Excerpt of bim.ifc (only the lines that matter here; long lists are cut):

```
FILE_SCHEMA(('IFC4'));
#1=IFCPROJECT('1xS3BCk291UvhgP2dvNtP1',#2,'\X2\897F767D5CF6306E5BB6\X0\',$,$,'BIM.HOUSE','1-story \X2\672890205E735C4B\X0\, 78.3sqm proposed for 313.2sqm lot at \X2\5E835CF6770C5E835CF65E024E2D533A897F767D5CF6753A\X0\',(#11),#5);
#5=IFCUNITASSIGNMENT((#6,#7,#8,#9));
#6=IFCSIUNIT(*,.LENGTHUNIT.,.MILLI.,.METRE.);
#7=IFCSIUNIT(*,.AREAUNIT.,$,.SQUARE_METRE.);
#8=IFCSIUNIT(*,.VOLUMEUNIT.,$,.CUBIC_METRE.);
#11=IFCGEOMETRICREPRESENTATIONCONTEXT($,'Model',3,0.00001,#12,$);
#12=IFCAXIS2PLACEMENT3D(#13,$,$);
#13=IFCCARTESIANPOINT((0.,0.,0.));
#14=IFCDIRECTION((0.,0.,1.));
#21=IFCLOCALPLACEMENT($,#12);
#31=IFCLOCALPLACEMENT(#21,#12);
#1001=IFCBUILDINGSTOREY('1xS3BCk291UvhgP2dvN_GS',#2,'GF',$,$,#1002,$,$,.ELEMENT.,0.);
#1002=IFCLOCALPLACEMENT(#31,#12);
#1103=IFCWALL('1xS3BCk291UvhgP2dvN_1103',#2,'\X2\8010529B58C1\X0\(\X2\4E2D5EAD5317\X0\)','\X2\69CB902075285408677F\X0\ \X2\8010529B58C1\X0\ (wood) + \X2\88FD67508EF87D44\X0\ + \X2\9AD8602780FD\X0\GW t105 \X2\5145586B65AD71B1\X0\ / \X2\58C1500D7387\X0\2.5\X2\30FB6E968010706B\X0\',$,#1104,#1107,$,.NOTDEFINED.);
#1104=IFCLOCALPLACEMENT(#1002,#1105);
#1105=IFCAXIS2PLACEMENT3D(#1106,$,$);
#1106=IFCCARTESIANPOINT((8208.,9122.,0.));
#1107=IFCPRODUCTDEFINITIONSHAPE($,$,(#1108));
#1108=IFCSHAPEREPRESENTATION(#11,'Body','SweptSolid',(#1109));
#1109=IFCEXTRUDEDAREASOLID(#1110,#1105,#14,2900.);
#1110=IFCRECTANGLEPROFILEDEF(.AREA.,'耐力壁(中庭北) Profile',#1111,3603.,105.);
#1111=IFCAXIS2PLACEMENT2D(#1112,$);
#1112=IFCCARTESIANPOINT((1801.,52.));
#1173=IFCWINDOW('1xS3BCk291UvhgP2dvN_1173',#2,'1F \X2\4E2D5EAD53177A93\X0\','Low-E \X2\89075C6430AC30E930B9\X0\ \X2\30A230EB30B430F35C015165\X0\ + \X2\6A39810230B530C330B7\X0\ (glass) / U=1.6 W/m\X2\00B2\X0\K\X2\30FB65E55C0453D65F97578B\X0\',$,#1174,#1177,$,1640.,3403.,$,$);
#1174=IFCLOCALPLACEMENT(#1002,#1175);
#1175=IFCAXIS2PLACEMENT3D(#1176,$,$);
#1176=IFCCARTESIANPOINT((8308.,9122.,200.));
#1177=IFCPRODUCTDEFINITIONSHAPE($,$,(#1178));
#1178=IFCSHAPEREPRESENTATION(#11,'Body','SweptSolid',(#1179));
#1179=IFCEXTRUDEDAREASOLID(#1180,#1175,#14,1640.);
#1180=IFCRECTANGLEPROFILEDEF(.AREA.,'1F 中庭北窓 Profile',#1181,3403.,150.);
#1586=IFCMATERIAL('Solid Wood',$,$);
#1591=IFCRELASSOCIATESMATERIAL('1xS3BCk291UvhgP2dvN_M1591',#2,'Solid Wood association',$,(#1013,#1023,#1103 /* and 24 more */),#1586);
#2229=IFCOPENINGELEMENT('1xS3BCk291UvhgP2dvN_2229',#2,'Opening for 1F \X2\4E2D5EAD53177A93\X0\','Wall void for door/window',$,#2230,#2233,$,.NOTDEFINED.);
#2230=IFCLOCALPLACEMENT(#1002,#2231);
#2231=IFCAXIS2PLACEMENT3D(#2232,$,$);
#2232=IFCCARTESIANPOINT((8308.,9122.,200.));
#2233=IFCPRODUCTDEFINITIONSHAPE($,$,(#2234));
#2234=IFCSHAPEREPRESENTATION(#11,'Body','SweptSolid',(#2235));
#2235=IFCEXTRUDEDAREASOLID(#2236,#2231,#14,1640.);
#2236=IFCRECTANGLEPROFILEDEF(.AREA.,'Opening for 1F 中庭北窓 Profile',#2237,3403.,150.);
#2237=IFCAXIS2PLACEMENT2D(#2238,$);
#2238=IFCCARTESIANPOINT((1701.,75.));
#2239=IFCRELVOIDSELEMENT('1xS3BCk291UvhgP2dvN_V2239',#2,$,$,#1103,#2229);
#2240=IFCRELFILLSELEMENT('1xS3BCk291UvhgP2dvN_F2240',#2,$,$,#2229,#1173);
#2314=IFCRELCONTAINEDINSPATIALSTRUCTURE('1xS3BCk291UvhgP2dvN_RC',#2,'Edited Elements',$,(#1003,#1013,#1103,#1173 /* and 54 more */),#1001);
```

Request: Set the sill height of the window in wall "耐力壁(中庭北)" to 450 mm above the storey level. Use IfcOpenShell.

```python
import numpy as np
import ifcopenshell
import ifcopenshell.api.geometry
import ifcopenshell.geom
import ifcopenshell.util.element
import ifcopenshell.util.placement
import ifcopenshell.util.shape
import ifcopenshell.util.unit

model = ifcopenshell.open("bim.ifc")
unit_scale = ifcopenshell.util.unit.calculate_unit_scale(model)

window = model.by_id(1173)
opening = window.FillsVoids[0].RelatingOpeningElement
storey = ifcopenshell.util.element.get_container(window, ifc_class="IfcBuildingStorey")
level = ifcopenshell.util.placement.get_local_placement(storey.ObjectPlacement)[2, 3]

# The opening's origin need not be at the sill, so measure its lowest point.
shape = ifcopenshell.geom.create_shape(ifcopenshell.geom.settings(), opening)
bottom = ifcopenshell.util.shape.get_shape_bottom_elevation(shape, shape.geometry) / unit_scale
dz = level + 0.45 / unit_scale - bottom

shift = np.array([0.0, 0.0, dz])
# The window is not placed relative to its opening, so move both.
for product in (opening, window):
    matrix = ifcopenshell.util.placement.get_local_placement(product.ObjectPlacement)
    matrix[:3, 3] += shift
    ifcopenshell.api.geometry.edit_object_placement(model, product=product, matrix=matrix, is_si=False)

print(f"moved by {dz * unit_scale:+.3f} m")

model.write("bim_updated.ifc")
```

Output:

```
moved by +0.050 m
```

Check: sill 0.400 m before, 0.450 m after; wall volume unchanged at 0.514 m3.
